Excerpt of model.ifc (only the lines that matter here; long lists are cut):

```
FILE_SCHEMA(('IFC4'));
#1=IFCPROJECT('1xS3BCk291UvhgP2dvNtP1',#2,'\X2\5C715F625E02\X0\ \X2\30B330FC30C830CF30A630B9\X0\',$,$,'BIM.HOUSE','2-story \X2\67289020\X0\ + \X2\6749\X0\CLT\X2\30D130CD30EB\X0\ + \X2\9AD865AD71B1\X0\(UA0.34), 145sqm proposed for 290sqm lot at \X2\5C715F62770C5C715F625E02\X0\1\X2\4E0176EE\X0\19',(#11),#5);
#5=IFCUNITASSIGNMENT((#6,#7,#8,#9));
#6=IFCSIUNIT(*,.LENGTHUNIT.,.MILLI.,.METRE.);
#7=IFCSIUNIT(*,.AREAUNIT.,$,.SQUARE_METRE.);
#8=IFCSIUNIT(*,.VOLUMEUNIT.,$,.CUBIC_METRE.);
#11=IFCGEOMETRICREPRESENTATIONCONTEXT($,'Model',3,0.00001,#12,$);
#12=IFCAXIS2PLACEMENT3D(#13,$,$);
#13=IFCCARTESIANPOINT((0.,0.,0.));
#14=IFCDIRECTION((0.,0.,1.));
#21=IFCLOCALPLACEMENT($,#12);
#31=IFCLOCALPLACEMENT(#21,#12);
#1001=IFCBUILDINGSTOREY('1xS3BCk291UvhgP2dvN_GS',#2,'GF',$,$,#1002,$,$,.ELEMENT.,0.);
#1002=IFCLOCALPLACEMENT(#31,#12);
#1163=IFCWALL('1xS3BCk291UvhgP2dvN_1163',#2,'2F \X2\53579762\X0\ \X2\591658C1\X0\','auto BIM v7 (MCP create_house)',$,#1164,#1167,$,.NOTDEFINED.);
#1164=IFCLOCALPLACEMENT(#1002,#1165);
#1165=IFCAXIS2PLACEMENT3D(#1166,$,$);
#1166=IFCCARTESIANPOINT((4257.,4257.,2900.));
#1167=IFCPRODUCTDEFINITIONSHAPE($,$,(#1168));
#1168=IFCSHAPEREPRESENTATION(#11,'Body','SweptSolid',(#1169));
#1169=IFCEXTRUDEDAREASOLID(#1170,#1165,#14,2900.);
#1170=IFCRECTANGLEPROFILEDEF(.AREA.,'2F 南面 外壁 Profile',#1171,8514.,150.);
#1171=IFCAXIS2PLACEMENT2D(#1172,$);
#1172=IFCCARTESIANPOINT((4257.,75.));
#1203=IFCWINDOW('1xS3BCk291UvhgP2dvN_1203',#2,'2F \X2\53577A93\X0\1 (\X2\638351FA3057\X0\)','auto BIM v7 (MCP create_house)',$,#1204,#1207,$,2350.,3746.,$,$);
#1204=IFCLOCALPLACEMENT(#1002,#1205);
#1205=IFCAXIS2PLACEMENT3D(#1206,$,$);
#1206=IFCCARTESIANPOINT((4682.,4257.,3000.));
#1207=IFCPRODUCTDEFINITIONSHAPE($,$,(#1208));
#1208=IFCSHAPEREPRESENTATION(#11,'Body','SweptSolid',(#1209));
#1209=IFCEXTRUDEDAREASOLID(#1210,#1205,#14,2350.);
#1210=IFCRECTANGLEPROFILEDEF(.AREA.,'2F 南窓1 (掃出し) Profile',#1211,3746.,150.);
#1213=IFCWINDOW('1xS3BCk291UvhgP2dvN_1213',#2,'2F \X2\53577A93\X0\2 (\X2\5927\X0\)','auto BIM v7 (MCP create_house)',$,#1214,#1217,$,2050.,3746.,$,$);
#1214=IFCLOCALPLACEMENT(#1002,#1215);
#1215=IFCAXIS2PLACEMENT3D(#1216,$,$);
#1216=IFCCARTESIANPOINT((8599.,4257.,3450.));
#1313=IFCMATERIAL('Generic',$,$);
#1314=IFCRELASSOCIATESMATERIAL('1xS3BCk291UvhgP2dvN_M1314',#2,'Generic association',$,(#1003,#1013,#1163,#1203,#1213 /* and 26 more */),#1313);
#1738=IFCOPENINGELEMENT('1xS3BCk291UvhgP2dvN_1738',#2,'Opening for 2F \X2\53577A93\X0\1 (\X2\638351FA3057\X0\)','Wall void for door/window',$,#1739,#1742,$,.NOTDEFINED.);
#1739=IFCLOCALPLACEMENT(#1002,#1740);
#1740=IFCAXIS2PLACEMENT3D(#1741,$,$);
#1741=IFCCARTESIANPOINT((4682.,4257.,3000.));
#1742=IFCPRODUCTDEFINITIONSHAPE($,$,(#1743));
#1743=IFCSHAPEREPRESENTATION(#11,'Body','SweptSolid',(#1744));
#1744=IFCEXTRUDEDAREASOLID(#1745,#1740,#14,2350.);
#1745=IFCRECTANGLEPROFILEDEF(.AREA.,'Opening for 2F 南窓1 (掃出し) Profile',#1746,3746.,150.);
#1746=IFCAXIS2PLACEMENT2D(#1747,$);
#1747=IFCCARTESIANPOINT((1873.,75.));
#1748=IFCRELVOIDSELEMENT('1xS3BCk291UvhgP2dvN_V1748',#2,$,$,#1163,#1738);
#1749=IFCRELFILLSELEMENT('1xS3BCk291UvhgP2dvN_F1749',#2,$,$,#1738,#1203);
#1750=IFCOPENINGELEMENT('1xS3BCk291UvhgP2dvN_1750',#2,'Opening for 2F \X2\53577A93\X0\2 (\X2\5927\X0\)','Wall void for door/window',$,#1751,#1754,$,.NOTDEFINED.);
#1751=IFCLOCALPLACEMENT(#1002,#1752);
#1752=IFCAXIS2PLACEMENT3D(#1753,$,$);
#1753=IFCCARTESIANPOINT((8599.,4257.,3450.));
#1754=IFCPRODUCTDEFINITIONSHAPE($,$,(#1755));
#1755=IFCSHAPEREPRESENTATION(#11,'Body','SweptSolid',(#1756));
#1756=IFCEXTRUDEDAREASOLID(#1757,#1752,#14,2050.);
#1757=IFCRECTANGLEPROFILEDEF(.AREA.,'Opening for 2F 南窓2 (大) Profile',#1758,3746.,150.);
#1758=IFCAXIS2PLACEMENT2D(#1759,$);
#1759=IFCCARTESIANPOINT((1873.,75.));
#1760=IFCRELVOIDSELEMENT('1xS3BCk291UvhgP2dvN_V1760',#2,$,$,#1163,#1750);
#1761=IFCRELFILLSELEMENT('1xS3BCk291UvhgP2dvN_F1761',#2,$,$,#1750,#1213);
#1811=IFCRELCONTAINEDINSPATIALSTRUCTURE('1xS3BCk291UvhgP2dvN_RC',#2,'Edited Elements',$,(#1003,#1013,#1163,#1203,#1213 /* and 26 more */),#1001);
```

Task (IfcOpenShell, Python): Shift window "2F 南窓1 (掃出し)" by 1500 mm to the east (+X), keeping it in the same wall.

```python
import ifcopenshell
import ifcopenshell.api.geometry
import ifcopenshell.util.placement

model = ifcopenshell.open("model.ifc")

window = model.by_guid("1xS3BCk291UvhgP2dvN_1203")
opening = window.FillsVoids[0].RelatingOpeningElement
wall = opening.VoidsElements[0].RelatingBuildingElement

wall_matrix = ifcopenshell.util.placement.get_local_placement(wall.ObjectPlacement)
shift = wall_matrix[:3, 0] * 1500.0
before = ifcopenshell.util.placement.get_local_placement(window.ObjectPlacement)[:3, 3].copy()

# The window is not placed relative to its opening, so move both.
for product in (opening, window):
    matrix = ifcopenshell.util.placement.get_local_placement(product.ObjectPlacement)
    matrix[:3, 3] += shift
    ifcopenshell.api.geometry.edit_object_placement(model, product=product, matrix=matrix, is_si=False)

after = ifcopenshell.util.placement.get_local_placement(window.ObjectPlacement)[:3, 3]
print("window moved by", (after - before).round(3) + 0.0)

model.write("model_rev.ifc")
```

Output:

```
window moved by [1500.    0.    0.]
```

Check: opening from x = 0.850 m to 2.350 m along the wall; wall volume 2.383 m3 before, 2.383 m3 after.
